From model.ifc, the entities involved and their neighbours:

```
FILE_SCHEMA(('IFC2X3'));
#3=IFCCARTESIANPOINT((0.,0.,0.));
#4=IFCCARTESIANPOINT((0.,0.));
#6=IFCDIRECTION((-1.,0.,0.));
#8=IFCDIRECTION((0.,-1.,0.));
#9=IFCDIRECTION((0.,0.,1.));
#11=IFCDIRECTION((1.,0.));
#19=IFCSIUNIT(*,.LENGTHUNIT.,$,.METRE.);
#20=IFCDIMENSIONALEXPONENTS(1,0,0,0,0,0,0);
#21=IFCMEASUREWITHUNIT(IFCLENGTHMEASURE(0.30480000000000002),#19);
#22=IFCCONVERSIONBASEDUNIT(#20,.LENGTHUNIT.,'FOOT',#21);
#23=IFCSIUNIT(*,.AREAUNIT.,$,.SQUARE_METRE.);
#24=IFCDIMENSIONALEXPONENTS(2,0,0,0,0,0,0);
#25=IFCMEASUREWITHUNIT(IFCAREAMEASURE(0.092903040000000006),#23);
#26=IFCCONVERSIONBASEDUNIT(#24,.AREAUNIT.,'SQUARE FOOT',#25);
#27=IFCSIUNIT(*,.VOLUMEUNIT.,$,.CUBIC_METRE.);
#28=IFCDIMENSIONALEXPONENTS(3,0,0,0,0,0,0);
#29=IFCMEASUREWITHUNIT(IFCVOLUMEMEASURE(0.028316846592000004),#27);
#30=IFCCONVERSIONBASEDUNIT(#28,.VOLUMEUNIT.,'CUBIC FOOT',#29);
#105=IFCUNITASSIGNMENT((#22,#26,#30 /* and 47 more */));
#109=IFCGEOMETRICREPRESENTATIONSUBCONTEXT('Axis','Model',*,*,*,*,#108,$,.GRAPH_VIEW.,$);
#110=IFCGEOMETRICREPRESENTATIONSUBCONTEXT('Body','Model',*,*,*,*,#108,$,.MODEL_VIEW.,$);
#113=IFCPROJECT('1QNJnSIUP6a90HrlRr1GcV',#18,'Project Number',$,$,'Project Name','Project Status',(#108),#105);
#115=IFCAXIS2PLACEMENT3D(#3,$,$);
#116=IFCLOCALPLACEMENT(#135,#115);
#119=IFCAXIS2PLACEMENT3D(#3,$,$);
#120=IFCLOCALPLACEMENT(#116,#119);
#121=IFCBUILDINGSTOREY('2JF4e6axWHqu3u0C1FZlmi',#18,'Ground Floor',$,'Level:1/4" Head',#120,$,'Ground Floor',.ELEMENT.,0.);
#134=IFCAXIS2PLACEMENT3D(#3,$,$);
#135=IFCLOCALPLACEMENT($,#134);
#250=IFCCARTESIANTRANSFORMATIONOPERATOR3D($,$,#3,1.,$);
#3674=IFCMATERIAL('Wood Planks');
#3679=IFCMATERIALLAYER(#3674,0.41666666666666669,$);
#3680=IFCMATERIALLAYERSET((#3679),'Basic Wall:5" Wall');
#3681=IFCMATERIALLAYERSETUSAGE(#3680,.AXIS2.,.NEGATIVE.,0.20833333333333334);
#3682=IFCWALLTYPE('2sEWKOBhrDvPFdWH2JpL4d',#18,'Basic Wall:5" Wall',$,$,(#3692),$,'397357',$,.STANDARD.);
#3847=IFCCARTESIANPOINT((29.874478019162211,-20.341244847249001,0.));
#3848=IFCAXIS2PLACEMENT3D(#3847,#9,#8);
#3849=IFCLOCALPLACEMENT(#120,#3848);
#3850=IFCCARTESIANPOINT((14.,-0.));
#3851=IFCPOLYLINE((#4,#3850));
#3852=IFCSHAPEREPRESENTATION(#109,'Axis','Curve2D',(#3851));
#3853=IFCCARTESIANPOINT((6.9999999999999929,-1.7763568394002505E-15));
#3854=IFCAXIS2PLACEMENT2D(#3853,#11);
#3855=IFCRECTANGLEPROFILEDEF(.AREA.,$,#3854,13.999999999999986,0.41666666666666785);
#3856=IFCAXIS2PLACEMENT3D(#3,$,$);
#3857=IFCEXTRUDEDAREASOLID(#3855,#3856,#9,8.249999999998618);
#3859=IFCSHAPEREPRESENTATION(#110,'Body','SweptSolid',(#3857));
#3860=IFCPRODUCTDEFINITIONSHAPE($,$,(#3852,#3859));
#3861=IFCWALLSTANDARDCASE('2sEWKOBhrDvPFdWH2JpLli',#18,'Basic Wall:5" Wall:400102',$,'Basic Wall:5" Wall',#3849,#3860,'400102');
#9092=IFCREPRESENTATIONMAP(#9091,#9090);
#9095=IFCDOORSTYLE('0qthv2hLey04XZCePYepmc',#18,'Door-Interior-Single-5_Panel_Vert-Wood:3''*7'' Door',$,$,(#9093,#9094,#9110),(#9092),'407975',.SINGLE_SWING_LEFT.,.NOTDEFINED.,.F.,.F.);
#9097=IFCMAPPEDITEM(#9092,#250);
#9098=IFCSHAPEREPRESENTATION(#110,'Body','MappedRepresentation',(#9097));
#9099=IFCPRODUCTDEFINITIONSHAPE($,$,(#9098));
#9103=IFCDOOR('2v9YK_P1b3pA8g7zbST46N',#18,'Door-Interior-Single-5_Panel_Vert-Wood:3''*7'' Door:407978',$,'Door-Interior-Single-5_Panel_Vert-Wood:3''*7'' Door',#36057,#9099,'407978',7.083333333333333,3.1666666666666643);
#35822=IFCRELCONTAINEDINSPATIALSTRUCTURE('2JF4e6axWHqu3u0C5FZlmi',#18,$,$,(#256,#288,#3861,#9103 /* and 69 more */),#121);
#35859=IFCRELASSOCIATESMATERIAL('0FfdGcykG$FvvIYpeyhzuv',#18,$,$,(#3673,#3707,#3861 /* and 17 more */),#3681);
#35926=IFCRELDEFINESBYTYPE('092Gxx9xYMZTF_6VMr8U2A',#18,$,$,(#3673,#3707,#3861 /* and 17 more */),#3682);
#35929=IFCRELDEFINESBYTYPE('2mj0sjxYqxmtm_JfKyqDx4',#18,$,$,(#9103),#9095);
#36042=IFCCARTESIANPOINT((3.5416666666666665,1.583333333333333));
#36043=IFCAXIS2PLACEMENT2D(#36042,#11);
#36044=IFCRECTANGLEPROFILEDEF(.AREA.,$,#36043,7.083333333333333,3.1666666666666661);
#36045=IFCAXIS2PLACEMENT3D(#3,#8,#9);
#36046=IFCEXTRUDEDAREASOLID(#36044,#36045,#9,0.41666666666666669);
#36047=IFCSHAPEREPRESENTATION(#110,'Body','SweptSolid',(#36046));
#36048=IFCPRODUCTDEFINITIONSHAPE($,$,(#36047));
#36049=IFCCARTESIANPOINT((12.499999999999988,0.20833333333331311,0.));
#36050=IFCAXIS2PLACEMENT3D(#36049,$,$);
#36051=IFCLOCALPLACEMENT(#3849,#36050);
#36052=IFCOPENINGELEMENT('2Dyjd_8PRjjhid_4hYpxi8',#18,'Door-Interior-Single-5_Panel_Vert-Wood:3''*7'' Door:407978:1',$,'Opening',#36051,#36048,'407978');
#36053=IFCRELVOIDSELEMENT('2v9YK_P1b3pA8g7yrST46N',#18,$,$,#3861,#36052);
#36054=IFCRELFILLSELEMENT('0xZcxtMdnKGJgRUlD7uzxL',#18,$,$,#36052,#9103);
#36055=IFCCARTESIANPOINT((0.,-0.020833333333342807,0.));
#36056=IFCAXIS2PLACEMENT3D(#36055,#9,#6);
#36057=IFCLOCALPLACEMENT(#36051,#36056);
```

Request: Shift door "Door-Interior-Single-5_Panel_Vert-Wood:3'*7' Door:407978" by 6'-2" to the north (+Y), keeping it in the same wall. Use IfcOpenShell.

```python
import ifcopenshell
import ifcopenshell.api.geometry
import ifcopenshell.util.placement
import ifcopenshell.util.unit

model = ifcopenshell.open("model.ifc")
unit_scale = ifcopenshell.util.unit.calculate_unit_scale(model)

door = model.by_guid("2v9YK_P1b3pA8g7zbST46N")
opening = door.FillsVoids[0].RelatingOpeningElement
wall = opening.VoidsElements[0].RelatingBuildingElement

wall_matrix = ifcopenshell.util.placement.get_local_placement(wall.ObjectPlacement)
shift = wall_matrix[:3, 0] * -74 * 0.0254 / unit_scale
before = ifcopenshell.util.placement.get_local_placement(door.ObjectPlacement)[:3, 3].copy()

# The door is placed relative to its opening, so it follows when the opening moves.
matrix = ifcopenshell.util.placement.get_local_placement(opening.ObjectPlacement)
matrix[:3, 3] += shift
ifcopenshell.api.geometry.edit_object_placement(
    model, product=opening, matrix=matrix, is_si=False, should_transform_children=True
)

after = ifcopenshell.util.placement.get_local_placement(door.ObjectPlacement)[:3, 3]
print("door moved by", (after - before).round(3) + 0.0)

model.write("model_v2.ifc")
```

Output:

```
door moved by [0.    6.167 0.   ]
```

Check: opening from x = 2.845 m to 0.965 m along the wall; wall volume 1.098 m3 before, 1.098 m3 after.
